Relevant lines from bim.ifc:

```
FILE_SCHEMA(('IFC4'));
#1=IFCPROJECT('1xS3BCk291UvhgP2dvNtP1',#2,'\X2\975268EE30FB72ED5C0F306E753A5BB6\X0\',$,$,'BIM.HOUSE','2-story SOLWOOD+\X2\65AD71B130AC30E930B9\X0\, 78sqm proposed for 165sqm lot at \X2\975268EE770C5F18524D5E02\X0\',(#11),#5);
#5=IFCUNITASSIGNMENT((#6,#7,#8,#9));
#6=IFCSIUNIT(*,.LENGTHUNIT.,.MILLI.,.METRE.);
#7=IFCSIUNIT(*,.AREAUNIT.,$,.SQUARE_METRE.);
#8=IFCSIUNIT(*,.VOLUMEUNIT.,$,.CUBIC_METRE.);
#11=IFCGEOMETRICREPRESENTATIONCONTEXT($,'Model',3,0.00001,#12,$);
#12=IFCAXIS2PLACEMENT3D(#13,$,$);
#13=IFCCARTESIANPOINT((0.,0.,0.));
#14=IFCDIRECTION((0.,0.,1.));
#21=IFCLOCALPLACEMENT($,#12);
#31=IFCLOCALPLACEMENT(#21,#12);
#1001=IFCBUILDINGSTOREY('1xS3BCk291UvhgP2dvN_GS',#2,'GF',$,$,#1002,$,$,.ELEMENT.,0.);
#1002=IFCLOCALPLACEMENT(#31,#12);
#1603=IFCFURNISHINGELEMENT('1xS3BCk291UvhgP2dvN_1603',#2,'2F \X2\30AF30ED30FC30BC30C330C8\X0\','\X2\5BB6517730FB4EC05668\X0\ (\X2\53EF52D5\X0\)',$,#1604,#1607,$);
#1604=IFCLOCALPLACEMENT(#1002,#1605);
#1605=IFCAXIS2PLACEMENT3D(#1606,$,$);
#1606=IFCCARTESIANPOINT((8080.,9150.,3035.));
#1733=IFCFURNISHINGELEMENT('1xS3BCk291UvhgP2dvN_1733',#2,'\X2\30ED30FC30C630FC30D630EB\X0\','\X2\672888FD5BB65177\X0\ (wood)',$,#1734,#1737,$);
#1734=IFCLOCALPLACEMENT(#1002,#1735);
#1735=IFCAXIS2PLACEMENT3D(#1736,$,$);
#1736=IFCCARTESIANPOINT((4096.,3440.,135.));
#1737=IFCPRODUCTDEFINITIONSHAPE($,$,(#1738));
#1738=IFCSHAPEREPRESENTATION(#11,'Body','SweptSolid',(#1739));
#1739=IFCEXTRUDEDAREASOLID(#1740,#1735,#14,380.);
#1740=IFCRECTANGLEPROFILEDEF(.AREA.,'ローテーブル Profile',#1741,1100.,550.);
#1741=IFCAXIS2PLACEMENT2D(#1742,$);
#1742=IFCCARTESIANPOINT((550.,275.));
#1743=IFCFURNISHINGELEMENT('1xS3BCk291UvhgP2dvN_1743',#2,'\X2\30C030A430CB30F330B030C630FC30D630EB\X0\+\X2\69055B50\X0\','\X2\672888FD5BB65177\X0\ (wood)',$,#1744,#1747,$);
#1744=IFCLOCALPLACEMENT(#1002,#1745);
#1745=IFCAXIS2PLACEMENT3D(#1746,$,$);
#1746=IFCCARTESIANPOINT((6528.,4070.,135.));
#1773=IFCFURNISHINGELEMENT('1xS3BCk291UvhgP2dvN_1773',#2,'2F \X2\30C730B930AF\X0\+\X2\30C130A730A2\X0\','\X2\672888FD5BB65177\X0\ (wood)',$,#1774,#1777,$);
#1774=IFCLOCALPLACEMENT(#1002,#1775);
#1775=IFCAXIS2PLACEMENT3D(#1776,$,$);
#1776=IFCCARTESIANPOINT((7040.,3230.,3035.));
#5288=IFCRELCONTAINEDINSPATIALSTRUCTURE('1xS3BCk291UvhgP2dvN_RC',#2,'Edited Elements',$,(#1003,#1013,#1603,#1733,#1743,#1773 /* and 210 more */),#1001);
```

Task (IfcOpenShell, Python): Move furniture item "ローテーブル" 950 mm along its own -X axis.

```python
import ifcopenshell
import ifcopenshell.api.geometry
import ifcopenshell.util.placement
import ifcopenshell.util.unit

model = ifcopenshell.open("bim.ifc")
unit_scale = ifcopenshell.util.unit.calculate_unit_scale(model)

item = model.by_id(1733)
matrix = ifcopenshell.util.placement.get_local_placement(item.ObjectPlacement)
matrix[:3, 3] -= matrix[:3, 0] * 0.95 / unit_scale
ifcopenshell.api.geometry.edit_object_placement(model, product=item, matrix=matrix, is_si=False)

print(ifcopenshell.util.placement.get_local_placement(item.ObjectPlacement).round(3) + 0.0)

model.write("bim_v2.ifc")
```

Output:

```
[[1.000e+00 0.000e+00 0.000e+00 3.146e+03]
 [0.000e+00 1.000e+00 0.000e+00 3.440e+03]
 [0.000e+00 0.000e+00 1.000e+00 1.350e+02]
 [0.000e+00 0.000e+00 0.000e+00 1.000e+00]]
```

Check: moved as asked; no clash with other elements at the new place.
